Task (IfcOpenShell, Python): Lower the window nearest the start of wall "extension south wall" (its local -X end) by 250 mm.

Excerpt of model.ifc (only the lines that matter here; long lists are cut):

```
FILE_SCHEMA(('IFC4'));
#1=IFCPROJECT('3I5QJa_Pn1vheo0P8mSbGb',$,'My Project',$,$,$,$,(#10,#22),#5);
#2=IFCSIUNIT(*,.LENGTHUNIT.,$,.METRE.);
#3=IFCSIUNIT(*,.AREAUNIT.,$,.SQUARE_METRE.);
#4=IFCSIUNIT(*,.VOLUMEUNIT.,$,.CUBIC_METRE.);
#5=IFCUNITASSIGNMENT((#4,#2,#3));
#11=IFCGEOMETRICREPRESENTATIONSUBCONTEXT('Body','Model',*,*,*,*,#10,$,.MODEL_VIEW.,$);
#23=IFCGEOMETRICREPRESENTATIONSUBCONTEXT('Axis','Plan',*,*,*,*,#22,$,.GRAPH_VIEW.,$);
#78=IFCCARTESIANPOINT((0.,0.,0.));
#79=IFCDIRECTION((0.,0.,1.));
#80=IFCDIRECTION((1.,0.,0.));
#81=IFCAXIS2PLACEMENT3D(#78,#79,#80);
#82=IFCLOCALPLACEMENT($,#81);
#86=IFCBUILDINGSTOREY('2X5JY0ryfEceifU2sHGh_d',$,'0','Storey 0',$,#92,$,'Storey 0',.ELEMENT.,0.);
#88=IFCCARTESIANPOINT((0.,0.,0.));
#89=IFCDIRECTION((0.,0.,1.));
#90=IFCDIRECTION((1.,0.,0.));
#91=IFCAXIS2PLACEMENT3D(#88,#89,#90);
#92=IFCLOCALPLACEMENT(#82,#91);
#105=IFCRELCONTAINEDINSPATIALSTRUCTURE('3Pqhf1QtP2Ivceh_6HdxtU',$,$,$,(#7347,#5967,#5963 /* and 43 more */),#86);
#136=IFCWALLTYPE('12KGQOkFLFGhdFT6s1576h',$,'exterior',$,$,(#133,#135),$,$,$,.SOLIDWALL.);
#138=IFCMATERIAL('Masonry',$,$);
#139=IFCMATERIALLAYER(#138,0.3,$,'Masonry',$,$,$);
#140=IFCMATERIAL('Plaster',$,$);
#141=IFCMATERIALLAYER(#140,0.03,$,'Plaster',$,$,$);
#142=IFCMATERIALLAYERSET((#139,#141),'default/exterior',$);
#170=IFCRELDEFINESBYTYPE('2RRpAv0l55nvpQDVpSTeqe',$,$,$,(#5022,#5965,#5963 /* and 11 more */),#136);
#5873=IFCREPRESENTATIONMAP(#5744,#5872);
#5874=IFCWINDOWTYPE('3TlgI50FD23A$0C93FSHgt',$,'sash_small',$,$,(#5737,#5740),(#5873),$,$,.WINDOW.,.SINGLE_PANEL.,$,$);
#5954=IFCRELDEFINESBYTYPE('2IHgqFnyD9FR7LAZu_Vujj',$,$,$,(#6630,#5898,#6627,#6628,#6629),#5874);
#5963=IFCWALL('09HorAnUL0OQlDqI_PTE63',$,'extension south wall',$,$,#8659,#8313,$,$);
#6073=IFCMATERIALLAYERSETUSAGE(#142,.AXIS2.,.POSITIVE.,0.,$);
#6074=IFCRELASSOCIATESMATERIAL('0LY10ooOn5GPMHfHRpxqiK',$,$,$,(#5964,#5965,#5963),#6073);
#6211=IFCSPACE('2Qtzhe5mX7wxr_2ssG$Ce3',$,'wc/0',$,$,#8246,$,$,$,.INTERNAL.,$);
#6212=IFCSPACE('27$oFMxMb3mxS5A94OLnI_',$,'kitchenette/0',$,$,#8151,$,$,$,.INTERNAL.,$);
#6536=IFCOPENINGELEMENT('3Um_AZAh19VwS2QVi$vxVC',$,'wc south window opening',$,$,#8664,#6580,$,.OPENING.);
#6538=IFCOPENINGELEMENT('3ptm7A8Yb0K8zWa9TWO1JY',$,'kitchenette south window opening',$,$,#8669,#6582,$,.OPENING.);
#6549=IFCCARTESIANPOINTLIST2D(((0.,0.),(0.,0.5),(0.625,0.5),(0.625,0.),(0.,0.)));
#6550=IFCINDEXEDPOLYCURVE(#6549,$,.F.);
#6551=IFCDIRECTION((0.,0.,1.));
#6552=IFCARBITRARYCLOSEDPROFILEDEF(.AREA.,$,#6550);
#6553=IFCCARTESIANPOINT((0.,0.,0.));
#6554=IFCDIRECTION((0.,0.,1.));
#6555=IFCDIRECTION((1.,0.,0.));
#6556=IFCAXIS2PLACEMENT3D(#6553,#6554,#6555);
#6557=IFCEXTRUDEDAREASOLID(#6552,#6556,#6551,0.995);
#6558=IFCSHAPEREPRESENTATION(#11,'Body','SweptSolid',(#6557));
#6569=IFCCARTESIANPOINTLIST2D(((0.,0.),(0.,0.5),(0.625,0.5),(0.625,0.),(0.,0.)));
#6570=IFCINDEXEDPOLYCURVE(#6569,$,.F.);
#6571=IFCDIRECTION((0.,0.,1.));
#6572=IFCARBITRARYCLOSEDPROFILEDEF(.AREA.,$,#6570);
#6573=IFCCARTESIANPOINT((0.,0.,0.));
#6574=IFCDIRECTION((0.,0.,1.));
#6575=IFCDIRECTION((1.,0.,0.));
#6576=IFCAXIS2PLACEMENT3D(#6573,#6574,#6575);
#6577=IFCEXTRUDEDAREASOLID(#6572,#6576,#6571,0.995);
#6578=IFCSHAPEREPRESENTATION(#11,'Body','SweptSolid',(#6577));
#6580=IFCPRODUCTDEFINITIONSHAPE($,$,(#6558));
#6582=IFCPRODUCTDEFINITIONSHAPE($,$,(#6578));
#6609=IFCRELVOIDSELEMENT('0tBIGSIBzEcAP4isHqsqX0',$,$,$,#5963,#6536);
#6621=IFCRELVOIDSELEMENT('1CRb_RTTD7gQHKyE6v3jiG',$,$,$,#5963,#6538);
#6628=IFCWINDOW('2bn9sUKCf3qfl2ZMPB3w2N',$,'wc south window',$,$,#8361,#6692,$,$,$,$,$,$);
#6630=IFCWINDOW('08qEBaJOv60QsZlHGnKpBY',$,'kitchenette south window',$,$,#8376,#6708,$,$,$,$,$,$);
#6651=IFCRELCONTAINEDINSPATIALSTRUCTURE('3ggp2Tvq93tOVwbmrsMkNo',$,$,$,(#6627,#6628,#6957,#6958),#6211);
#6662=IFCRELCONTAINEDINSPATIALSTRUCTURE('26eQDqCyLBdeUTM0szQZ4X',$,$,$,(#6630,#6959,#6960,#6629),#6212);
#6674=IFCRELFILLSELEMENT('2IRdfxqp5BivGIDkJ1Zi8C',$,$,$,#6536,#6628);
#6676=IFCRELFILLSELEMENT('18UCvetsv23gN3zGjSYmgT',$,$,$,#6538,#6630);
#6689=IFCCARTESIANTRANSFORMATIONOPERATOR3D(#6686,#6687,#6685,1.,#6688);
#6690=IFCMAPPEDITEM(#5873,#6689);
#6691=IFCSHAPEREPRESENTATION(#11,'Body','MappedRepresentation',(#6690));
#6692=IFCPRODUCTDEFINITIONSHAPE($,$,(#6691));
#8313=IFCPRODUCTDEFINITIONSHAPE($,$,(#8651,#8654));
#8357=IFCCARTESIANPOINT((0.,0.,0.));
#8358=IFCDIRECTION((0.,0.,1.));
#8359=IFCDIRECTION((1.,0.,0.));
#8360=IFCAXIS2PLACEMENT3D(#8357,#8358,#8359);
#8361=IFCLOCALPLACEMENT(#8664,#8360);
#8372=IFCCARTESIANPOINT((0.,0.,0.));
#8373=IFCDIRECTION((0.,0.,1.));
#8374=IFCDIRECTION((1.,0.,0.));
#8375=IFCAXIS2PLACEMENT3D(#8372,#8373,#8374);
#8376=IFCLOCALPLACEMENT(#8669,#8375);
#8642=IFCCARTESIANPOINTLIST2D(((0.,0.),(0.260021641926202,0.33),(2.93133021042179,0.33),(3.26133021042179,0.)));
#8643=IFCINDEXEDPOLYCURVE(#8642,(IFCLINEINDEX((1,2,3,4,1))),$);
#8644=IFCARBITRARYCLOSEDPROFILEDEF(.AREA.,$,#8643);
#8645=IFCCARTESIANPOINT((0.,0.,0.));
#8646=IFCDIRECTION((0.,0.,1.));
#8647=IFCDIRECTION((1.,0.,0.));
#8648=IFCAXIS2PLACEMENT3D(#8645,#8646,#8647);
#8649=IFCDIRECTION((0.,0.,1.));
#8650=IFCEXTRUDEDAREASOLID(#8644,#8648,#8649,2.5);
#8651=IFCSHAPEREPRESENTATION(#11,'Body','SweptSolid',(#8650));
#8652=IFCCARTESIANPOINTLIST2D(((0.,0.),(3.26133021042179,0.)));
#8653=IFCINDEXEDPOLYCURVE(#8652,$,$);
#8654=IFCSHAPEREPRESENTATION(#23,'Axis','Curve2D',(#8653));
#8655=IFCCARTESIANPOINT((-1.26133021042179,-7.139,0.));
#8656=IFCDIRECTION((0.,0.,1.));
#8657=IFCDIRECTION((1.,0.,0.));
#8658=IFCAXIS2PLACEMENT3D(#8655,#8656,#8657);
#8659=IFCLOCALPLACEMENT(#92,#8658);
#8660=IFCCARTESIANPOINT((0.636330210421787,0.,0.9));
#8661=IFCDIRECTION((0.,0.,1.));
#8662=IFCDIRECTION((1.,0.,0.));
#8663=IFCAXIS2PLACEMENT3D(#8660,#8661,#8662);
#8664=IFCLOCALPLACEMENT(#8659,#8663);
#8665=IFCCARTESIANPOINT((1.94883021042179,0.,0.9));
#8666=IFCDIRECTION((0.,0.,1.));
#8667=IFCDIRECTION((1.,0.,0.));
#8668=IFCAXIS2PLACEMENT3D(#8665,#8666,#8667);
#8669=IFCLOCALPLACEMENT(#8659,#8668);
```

```python
import numpy as np
import ifcopenshell
import ifcopenshell.api.geometry
import ifcopenshell.util.placement
import ifcopenshell.util.unit

model = ifcopenshell.open("model.ifc")
unit_scale = ifcopenshell.util.unit.calculate_unit_scale(model)

window = model.by_guid("2bn9sUKCf3qfl2ZMPB3w2N")
opening = window.FillsVoids[0].RelatingOpeningElement
dz = -0.25 / unit_scale

shift = np.array([0.0, 0.0, dz])
# The window is placed relative to its opening, so it follows when the opening moves.
matrix = ifcopenshell.util.placement.get_local_placement(opening.ObjectPlacement)
matrix[:3, 3] += shift
ifcopenshell.api.geometry.edit_object_placement(
    model, product=opening, matrix=matrix, is_si=False, should_transform_children=True
)

print(f"moved by {dz * unit_scale:+.3f} m")

model.write("model_edited.ifc")
```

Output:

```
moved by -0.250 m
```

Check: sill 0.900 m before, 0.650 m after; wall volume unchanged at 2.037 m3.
